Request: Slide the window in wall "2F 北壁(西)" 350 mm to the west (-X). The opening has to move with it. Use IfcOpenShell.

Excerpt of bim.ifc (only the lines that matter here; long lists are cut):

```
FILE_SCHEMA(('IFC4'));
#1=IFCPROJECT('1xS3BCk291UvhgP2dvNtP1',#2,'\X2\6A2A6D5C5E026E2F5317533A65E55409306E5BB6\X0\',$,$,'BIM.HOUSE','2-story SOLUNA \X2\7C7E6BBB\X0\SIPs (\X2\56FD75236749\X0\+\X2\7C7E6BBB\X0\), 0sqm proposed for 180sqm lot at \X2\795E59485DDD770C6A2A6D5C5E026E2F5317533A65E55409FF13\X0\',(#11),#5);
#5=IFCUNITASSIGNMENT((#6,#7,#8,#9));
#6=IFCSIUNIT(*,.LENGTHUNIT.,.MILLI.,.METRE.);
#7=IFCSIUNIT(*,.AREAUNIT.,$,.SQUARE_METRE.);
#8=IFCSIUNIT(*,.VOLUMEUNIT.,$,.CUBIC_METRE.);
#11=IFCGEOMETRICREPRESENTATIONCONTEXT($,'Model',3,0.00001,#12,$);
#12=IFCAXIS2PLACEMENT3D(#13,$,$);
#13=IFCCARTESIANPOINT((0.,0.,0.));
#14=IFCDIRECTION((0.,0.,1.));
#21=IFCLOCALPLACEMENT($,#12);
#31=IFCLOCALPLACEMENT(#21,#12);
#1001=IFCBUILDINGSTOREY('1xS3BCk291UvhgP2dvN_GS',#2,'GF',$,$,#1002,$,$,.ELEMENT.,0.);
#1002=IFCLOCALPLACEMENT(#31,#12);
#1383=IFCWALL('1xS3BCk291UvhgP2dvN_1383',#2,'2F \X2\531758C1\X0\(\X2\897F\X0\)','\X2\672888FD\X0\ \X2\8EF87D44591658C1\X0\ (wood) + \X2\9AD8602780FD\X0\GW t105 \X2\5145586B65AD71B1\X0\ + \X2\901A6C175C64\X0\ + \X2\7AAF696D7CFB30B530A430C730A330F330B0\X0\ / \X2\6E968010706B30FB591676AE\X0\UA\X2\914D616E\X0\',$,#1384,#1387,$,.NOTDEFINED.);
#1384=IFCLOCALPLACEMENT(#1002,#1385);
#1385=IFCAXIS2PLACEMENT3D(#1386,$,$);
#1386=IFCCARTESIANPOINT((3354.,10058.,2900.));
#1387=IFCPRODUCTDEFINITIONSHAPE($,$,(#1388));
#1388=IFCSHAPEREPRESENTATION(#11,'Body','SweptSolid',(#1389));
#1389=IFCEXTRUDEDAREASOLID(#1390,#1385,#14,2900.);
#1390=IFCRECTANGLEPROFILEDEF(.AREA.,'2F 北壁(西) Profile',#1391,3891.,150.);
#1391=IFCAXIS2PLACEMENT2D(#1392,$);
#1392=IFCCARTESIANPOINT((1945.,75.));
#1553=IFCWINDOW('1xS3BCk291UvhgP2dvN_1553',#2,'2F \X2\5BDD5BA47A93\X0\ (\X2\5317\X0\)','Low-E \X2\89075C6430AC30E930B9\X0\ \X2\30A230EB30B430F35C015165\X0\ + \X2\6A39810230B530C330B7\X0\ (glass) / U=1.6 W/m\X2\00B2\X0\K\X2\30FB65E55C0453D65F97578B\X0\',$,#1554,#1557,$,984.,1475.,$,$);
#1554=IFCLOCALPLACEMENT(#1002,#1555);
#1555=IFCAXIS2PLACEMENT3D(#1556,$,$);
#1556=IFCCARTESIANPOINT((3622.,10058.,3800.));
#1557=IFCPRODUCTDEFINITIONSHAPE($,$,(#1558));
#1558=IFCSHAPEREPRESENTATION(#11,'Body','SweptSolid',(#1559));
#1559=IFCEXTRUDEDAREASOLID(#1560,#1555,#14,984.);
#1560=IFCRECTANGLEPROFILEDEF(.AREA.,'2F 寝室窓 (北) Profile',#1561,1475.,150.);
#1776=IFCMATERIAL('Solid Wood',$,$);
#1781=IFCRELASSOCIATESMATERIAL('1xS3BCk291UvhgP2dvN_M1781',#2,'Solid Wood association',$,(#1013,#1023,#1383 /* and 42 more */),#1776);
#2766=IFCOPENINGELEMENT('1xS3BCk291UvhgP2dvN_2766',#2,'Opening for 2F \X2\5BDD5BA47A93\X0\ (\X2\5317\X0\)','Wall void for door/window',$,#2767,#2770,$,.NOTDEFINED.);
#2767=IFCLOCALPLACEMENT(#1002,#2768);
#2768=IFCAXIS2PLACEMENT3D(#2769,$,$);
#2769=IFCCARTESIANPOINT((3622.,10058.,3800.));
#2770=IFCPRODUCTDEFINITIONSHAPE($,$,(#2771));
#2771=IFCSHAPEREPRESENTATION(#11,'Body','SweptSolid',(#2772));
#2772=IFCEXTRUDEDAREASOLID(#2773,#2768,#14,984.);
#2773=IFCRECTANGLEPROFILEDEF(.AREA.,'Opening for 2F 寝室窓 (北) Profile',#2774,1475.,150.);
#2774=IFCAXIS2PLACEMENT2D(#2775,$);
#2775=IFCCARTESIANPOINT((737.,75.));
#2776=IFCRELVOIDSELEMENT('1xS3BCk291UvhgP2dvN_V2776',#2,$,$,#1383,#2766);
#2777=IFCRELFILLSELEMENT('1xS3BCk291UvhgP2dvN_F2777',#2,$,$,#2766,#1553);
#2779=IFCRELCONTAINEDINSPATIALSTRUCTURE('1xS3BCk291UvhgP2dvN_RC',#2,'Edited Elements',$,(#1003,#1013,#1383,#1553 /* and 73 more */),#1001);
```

```python
import ifcopenshell
import ifcopenshell.api.geometry
import ifcopenshell.util.placement
import ifcopenshell.util.unit

model = ifcopenshell.open("bim.ifc")
unit_scale = ifcopenshell.util.unit.calculate_unit_scale(model)

window = model.by_guid("1xS3BCk291UvhgP2dvN_1553")
opening = window.FillsVoids[0].RelatingOpeningElement
wall = opening.VoidsElements[0].RelatingBuildingElement

wall_matrix = ifcopenshell.util.placement.get_local_placement(wall.ObjectPlacement)
shift = wall_matrix[:3, 0] * -0.35 / unit_scale
before = ifcopenshell.util.placement.get_local_placement(window.ObjectPlacement)[:3, 3].copy()

# The window is not placed relative to its opening, so move both.
for product in (opening, window):
    matrix = ifcopenshell.util.placement.get_local_placement(product.ObjectPlacement)
    matrix[:3, 3] += shift
    ifcopenshell.api.geometry.edit_object_placement(model, product=product, matrix=matrix, is_si=False)

after = ifcopenshell.util.placement.get_local_placement(window.ObjectPlacement)[:3, 3]
print("window moved by", (after - before).round(3) + 0.0)

model.write("bim_v2.ifc")
```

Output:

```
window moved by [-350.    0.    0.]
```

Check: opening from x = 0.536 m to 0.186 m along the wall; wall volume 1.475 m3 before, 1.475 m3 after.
